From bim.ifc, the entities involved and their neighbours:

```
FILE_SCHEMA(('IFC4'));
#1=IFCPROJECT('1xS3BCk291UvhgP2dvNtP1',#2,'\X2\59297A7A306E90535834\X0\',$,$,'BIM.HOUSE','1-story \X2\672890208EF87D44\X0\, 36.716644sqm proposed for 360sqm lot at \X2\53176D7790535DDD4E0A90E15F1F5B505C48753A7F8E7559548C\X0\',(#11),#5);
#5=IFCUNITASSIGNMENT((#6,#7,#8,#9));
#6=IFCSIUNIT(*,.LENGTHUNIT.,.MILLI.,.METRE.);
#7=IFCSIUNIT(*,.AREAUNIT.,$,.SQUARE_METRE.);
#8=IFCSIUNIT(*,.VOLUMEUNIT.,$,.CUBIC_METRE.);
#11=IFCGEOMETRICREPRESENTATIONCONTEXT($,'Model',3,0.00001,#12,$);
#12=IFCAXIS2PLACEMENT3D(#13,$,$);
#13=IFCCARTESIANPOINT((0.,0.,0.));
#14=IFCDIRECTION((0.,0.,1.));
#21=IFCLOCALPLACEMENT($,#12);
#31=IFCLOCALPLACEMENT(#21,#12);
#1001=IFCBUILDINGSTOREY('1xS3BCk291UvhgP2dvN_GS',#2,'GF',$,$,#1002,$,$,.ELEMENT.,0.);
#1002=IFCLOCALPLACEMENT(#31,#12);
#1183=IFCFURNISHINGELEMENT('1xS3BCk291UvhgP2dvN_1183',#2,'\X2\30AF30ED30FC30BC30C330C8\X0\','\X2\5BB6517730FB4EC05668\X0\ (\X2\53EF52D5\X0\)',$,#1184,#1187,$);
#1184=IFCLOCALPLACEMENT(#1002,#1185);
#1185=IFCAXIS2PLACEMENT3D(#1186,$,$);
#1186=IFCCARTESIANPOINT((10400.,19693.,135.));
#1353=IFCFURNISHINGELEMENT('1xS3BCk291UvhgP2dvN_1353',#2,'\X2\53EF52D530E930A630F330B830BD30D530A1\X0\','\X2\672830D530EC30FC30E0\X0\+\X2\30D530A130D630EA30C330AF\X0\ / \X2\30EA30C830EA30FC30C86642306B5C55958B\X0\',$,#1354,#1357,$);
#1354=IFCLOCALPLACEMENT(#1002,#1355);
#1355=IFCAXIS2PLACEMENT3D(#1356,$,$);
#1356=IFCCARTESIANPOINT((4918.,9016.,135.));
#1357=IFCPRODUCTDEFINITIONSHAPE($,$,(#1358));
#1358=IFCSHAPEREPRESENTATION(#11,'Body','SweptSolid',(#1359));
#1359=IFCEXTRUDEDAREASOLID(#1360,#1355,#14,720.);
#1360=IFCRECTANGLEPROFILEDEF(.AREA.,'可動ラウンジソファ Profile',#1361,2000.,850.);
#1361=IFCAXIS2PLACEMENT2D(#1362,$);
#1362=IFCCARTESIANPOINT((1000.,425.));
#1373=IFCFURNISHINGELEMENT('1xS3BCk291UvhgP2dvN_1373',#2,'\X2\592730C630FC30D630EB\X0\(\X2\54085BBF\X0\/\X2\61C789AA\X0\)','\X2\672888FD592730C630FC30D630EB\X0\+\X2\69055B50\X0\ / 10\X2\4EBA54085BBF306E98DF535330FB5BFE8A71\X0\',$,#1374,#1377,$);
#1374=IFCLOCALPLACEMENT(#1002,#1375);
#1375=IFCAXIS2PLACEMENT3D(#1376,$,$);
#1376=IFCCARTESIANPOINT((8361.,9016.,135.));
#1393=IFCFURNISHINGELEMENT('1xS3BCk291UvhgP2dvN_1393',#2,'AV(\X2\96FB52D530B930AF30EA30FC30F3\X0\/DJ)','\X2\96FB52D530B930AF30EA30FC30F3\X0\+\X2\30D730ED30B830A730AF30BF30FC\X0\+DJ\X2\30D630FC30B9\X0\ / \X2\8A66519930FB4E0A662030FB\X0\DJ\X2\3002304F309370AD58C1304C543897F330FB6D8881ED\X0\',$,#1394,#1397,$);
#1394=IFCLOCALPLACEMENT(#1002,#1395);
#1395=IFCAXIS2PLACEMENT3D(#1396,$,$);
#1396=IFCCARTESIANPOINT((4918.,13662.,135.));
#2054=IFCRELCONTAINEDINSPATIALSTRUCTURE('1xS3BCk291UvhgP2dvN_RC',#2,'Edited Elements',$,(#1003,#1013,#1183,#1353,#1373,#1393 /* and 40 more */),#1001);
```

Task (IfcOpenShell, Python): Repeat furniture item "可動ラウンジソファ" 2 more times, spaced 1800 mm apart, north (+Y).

```python
import numpy as np
import ifcopenshell
import ifcopenshell.api.geometry
import ifcopenshell.api.root
import ifcopenshell.util.element
import ifcopenshell.util.placement

model = ifcopenshell.open("bim.ifc")


def reuse_history(source, copy):
    """copy_class also copies each property set's owner history, people and application; keep the originals."""
    for rel in copy.IsDefinedBy:
        if rel.is_a("IfcRelDefinesByProperties") and (history := rel.RelatingPropertyDefinition.OwnerHistory):
            rel.RelatingPropertyDefinition.OwnerHistory = source.OwnerHistory
            ifcopenshell.util.element.remove_deep2(model, history)


source = model.by_guid("1xS3BCk291UvhgP2dvN_1353")
base = ifcopenshell.util.placement.get_local_placement(source.ObjectPlacement)
step = np.array([0.0, 1.0, 0.0]) * 1800.0

for i in range(1, 3):
    copy = ifcopenshell.api.root.copy_class(model, product=source)
    copy.Representation = ifcopenshell.util.element.copy_deep(
        model, source.Representation, exclude=["IfcGeometricRepresentationContext", "IfcRepresentationMap"]
    )
    reuse_history(source, copy)
    matrix = base.copy()
    matrix[:3, 3] += i * step
    print("added at", matrix[:3, 3].round(3) + 0.0)
    ifcopenshell.api.geometry.edit_object_placement(model, product=copy, matrix=matrix, is_si=False)

model.write("bim_edited.ifc")
```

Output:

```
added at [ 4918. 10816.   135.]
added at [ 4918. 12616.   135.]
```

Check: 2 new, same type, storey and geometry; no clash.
